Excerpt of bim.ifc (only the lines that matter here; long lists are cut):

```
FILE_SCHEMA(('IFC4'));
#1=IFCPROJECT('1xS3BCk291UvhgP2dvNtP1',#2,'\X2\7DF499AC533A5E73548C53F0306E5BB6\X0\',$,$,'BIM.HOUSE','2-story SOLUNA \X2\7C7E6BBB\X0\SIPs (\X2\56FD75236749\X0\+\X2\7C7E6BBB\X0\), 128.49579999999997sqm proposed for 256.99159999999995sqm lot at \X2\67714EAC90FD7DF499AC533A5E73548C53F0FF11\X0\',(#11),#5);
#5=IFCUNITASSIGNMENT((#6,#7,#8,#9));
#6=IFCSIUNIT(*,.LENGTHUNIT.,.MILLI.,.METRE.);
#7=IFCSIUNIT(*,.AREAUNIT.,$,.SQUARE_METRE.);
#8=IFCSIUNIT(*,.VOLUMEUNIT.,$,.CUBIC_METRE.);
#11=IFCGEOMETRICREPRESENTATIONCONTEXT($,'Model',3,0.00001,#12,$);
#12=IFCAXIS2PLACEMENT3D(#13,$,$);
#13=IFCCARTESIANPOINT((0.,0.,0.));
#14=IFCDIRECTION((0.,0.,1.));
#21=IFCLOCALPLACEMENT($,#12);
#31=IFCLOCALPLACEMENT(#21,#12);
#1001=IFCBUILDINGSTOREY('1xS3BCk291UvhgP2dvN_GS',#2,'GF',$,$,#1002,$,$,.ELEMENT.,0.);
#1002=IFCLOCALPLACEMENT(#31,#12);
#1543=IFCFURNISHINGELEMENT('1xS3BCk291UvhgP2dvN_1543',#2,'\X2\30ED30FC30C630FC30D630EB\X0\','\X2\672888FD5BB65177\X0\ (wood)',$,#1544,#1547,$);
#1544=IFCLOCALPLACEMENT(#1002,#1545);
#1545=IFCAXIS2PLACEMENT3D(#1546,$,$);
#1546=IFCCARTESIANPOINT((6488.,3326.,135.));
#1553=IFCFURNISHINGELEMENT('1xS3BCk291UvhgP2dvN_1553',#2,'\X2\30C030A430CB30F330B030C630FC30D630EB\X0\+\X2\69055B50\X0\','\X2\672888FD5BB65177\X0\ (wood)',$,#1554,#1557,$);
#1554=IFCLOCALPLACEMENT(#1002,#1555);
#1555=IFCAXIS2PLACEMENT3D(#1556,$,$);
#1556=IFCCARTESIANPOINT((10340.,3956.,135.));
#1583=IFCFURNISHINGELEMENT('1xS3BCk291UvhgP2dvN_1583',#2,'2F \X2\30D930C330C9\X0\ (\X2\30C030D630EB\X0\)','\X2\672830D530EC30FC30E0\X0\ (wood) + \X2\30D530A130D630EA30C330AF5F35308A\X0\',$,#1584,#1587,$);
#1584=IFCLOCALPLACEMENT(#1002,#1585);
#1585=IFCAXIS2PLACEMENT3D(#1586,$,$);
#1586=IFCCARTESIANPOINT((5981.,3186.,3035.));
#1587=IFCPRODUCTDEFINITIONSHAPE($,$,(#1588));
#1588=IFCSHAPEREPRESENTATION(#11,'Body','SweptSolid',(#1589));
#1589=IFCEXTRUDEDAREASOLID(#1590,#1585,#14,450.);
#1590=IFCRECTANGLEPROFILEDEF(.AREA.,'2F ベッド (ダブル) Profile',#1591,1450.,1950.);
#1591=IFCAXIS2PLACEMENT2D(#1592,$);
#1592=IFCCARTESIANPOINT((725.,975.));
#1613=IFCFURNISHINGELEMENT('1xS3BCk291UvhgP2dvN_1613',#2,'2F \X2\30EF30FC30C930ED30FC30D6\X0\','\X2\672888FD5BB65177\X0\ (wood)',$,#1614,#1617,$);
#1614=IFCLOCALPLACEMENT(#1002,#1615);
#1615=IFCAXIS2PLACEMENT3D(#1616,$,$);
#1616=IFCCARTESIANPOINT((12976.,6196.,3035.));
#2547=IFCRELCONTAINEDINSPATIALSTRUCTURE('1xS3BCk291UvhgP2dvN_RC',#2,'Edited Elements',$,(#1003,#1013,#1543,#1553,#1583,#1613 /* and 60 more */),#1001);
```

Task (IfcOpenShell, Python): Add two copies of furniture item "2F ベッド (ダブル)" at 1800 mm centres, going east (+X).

```python
import numpy as np
import ifcopenshell
import ifcopenshell.api.geometry
import ifcopenshell.api.root
import ifcopenshell.util.element
import ifcopenshell.util.placement
import ifcopenshell.util.unit

model = ifcopenshell.open("bim.ifc")
unit_scale = ifcopenshell.util.unit.calculate_unit_scale(model)


def reuse_history(source, copy):
    """copy_class also copies each property set's owner history, people and application; keep the originals."""
    for rel in copy.IsDefinedBy:
        if rel.is_a("IfcRelDefinesByProperties") and (history := rel.RelatingPropertyDefinition.OwnerHistory):
            rel.RelatingPropertyDefinition.OwnerHistory = source.OwnerHistory
            ifcopenshell.util.element.remove_deep2(model, history)


source = model.by_id(1583)
base = ifcopenshell.util.placement.get_local_placement(source.ObjectPlacement)
step = np.array([1.0, 0.0, 0.0]) * 1.8 / unit_scale

for i in range(1, 3):
    copy = ifcopenshell.api.root.copy_class(model, product=source)
    copy.Representation = ifcopenshell.util.element.copy_deep(
        model, source.Representation, exclude=["IfcGeometricRepresentationContext", "IfcRepresentationMap"]
    )
    reuse_history(source, copy)
    matrix = base.copy()
    matrix[:3, 3] += i * step
    print("added at", matrix[:3, 3].round(3) + 0.0)
    ifcopenshell.api.geometry.edit_object_placement(model, product=copy, matrix=matrix, is_si=False)

model.write("bim_updated.ifc")
```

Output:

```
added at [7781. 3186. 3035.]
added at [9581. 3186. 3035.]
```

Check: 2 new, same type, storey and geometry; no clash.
